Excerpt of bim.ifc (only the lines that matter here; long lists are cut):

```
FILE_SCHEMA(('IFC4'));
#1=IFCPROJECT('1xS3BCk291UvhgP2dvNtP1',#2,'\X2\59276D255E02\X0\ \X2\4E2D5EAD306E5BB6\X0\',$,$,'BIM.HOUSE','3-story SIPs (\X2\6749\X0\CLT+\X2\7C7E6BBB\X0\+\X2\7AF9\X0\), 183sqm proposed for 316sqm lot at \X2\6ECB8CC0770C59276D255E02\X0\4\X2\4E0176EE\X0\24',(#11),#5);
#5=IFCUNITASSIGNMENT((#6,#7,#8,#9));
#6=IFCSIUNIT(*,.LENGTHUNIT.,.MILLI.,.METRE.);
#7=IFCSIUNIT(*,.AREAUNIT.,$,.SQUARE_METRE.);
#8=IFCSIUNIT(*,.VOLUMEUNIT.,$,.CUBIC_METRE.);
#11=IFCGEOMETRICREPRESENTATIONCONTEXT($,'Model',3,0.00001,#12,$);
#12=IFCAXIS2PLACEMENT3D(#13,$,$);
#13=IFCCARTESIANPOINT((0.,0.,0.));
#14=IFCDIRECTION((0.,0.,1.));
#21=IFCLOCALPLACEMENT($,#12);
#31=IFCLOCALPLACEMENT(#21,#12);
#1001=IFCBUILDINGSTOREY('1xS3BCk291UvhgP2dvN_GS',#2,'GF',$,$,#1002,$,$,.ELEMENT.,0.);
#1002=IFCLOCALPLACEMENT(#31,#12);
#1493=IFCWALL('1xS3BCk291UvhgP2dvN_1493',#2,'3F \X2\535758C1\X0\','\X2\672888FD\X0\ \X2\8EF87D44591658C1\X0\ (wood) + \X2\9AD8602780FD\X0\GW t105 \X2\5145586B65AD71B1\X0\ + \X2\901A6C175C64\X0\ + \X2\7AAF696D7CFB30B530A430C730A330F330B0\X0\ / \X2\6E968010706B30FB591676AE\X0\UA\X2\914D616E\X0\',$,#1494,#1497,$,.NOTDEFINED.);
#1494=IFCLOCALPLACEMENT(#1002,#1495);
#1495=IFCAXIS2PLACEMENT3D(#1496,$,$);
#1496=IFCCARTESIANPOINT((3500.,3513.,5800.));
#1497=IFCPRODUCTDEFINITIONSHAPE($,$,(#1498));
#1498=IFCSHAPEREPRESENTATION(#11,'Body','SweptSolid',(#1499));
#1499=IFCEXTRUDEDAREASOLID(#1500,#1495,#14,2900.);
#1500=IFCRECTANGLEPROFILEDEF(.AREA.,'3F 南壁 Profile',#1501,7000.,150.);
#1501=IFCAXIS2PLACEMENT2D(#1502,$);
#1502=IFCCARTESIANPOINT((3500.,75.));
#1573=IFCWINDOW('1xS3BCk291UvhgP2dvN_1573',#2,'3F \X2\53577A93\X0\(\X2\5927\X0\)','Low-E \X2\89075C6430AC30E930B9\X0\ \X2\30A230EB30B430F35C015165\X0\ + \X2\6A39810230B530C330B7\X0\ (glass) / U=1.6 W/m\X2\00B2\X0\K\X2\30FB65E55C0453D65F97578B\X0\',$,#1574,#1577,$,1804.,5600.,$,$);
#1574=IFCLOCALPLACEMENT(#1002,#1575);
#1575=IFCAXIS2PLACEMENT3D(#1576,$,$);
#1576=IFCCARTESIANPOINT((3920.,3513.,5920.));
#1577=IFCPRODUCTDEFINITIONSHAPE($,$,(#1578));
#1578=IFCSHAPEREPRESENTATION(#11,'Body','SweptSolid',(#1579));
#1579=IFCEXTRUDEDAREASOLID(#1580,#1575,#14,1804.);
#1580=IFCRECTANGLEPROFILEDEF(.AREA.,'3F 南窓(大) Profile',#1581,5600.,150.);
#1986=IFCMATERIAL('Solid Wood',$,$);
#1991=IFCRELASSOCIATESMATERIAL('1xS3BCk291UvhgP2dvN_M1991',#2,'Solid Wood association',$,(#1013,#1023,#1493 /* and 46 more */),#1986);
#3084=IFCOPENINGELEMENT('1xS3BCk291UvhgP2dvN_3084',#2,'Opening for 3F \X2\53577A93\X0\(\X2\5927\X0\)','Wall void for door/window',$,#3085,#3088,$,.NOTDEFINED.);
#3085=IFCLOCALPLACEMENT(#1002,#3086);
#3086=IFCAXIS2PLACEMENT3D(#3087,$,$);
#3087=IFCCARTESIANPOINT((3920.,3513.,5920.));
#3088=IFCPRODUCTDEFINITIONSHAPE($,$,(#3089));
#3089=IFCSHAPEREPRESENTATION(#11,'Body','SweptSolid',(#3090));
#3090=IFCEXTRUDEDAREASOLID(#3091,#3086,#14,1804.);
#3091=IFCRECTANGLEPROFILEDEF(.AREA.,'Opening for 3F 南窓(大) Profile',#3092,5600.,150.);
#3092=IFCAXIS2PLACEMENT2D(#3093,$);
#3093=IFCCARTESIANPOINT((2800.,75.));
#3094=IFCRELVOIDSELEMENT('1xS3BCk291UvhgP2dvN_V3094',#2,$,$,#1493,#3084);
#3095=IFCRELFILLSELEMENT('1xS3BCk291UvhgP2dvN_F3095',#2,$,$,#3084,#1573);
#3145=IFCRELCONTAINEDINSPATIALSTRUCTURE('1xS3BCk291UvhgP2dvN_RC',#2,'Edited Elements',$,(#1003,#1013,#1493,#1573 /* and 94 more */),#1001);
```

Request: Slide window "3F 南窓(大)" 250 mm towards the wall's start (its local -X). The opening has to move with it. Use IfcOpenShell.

```python
import ifcopenshell
import ifcopenshell.api.geometry
import ifcopenshell.util.placement
import ifcopenshell.util.unit

model = ifcopenshell.open("bim.ifc")
unit_scale = ifcopenshell.util.unit.calculate_unit_scale(model)

window = model.by_guid("1xS3BCk291UvhgP2dvN_1573")
opening = window.FillsVoids[0].RelatingOpeningElement
wall = opening.VoidsElements[0].RelatingBuildingElement

wall_matrix = ifcopenshell.util.placement.get_local_placement(wall.ObjectPlacement)
shift = wall_matrix[:3, 0] * -0.25 / unit_scale
before = ifcopenshell.util.placement.get_local_placement(window.ObjectPlacement)[:3, 3].copy()

# The window is not placed relative to its opening, so move both.
for product in (opening, window):
    matrix = ifcopenshell.util.placement.get_local_placement(product.ObjectPlacement)
    matrix[:3, 3] += shift
    ifcopenshell.api.geometry.edit_object_placement(model, product=product, matrix=matrix, is_si=False)

after = ifcopenshell.util.placement.get_local_placement(window.ObjectPlacement)[:3, 3]
print("window moved by", (after - before).round(3) + 0.0)

model.write("bim_rev.ifc")
```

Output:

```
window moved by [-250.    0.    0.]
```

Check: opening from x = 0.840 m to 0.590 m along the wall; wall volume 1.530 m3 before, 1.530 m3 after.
